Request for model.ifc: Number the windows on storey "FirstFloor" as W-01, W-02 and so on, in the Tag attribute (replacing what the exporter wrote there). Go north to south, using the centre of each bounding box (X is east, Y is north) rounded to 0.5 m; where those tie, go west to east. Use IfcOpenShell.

First a look at what the model holds.

```python
import ifcopenshell
import ifcopenshell.util.element
import ifcopenshell.util.placement

model = ifcopenshell.open("model.ifc")
print(model.schema)
storey = next(s for s in model.by_type("IfcBuildingStorey") if s.Name == "FirstFloor")
windows = [e for e in ifcopenshell.util.element.get_decomposition(storey) if e.is_a("IfcWindow")]
for e in sorted(windows, key=lambda e: e.id()):
    origin = ifcopenshell.util.placement.get_local_placement(e.ObjectPlacement)[:3, 3]
    print(e.id(), e.Tag, e.Name, origin.round(2) + 0.0, sep=" | ")
```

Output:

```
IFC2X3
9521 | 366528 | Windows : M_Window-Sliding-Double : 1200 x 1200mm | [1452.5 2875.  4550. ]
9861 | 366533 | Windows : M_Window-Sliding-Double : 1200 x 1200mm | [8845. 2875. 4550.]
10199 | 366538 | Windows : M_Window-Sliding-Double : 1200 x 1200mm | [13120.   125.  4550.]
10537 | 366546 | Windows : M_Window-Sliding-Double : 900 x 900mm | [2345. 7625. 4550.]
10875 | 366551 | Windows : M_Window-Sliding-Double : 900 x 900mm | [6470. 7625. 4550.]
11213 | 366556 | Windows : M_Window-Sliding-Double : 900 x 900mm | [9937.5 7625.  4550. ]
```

```python
import ifcopenshell
import ifcopenshell.geom
import ifcopenshell.util.element
import ifcopenshell.util.shape

model = ifcopenshell.open("model.ifc")
settings = ifcopenshell.geom.settings()
settings.set("use-world-coords", True)


def centre(element):
    shape = ifcopenshell.geom.create_shape(settings, element)
    return ifcopenshell.util.shape.get_bbox_centroid(shape.geometry)


storey = next(s for s in model.by_type("IfcBuildingStorey") if s.Name == "FirstFloor")
windows = [e for e in ifcopenshell.util.element.get_decomposition(storey) if e.is_a("IfcWindow")]

# Insertion points can sit at a corner or the storey origin, so sort by the geometry (in metres).
centres = {e: centre(e) for e in windows}
windows.sort(key=lambda e: (-round(centres[e][1] / 0.5), centres[e][0]))

for i, e in enumerate(windows, start=1):
    number = f"W-{i:02d}"
    e.Tag = number
    print(e.id(), number)

model.write("model_updated.ifc")
```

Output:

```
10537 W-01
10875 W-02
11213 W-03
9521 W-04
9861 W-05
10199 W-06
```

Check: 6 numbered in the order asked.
